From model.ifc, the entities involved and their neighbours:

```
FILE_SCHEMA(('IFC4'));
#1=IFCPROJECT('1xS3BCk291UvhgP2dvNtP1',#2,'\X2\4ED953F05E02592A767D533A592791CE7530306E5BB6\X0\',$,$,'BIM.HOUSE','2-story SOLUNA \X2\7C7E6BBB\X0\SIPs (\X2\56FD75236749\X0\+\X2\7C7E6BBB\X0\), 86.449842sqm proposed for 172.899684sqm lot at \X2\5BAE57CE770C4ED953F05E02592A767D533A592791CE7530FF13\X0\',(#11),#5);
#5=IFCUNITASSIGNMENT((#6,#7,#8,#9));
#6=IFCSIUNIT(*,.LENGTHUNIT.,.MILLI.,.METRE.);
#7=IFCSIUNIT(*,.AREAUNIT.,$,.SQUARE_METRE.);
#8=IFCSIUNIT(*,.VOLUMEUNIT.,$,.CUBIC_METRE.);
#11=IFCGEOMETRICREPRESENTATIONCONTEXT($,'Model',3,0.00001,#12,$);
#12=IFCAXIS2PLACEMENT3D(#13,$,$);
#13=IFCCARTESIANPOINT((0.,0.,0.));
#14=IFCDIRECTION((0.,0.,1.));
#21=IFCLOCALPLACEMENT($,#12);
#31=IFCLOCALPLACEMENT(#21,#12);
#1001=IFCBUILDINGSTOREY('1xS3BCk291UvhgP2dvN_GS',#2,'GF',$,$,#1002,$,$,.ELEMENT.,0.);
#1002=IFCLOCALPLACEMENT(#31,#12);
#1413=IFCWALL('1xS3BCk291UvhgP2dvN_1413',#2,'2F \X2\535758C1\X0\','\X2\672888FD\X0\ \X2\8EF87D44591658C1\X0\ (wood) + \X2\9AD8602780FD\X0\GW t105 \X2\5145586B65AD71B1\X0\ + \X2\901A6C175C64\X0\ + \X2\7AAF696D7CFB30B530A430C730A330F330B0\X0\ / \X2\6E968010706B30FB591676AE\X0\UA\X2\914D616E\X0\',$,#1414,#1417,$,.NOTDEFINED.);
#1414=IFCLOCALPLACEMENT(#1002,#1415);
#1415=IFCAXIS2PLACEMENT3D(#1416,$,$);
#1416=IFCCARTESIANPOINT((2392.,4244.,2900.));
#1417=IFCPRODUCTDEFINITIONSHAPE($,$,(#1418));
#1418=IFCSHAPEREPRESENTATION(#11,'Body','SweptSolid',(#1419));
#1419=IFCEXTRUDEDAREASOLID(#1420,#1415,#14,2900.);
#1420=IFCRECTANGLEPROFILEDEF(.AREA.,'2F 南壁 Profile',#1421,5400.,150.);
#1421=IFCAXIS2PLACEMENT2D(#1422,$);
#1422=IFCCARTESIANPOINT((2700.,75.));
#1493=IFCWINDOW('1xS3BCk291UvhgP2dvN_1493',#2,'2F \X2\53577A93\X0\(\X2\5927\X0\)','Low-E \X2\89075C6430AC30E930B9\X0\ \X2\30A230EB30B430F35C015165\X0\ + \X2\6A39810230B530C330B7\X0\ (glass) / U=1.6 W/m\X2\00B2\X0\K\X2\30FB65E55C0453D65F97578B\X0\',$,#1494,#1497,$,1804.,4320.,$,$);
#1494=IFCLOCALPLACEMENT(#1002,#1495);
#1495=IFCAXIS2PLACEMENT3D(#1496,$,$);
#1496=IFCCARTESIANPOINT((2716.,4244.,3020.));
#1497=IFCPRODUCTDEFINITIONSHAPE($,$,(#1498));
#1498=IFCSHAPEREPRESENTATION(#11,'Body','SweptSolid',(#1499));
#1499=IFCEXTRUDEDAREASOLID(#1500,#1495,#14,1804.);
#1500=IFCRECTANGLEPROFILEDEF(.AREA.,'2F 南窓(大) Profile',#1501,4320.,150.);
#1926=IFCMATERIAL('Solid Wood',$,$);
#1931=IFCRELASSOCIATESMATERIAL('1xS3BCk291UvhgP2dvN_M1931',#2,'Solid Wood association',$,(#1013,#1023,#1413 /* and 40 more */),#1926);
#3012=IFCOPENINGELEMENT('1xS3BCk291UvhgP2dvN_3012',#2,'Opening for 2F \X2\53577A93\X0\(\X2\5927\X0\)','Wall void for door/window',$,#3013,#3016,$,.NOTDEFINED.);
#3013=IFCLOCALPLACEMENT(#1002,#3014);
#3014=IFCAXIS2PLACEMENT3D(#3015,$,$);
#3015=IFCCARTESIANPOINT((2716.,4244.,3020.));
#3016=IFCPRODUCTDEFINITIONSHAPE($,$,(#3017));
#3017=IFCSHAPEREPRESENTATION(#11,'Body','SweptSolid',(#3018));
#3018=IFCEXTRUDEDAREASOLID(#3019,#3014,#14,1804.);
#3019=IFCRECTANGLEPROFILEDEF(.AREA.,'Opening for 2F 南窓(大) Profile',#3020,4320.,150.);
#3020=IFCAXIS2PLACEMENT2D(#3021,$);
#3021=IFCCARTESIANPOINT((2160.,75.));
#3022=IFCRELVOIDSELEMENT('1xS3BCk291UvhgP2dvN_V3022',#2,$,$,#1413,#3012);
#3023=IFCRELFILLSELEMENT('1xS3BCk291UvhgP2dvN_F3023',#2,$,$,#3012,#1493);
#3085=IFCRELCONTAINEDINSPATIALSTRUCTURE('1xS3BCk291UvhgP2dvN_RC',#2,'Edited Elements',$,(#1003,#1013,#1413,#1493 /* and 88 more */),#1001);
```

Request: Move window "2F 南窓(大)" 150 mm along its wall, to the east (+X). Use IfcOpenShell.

```python
import ifcopenshell
import ifcopenshell.api.geometry
import ifcopenshell.util.placement

model = ifcopenshell.open("model.ifc")

window = model.by_guid("1xS3BCk291UvhgP2dvN_1493")
opening = window.FillsVoids[0].RelatingOpeningElement
wall = opening.VoidsElements[0].RelatingBuildingElement

wall_matrix = ifcopenshell.util.placement.get_local_placement(wall.ObjectPlacement)
shift = wall_matrix[:3, 0] * 150.0
before = ifcopenshell.util.placement.get_local_placement(window.ObjectPlacement)[:3, 3].copy()

# The window is not placed relative to its opening, so move both.
for product in (opening, window):
    matrix = ifcopenshell.util.placement.get_local_placement(product.ObjectPlacement)
    matrix[:3, 3] += shift
    ifcopenshell.api.geometry.edit_object_placement(model, product=product, matrix=matrix, is_si=False)

after = ifcopenshell.util.placement.get_local_placement(window.ObjectPlacement)[:3, 3]
print("window moved by", (after - before).round(3) + 0.0)

model.write("model_rev.ifc")
```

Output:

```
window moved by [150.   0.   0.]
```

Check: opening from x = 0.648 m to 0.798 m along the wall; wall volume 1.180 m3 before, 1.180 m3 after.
